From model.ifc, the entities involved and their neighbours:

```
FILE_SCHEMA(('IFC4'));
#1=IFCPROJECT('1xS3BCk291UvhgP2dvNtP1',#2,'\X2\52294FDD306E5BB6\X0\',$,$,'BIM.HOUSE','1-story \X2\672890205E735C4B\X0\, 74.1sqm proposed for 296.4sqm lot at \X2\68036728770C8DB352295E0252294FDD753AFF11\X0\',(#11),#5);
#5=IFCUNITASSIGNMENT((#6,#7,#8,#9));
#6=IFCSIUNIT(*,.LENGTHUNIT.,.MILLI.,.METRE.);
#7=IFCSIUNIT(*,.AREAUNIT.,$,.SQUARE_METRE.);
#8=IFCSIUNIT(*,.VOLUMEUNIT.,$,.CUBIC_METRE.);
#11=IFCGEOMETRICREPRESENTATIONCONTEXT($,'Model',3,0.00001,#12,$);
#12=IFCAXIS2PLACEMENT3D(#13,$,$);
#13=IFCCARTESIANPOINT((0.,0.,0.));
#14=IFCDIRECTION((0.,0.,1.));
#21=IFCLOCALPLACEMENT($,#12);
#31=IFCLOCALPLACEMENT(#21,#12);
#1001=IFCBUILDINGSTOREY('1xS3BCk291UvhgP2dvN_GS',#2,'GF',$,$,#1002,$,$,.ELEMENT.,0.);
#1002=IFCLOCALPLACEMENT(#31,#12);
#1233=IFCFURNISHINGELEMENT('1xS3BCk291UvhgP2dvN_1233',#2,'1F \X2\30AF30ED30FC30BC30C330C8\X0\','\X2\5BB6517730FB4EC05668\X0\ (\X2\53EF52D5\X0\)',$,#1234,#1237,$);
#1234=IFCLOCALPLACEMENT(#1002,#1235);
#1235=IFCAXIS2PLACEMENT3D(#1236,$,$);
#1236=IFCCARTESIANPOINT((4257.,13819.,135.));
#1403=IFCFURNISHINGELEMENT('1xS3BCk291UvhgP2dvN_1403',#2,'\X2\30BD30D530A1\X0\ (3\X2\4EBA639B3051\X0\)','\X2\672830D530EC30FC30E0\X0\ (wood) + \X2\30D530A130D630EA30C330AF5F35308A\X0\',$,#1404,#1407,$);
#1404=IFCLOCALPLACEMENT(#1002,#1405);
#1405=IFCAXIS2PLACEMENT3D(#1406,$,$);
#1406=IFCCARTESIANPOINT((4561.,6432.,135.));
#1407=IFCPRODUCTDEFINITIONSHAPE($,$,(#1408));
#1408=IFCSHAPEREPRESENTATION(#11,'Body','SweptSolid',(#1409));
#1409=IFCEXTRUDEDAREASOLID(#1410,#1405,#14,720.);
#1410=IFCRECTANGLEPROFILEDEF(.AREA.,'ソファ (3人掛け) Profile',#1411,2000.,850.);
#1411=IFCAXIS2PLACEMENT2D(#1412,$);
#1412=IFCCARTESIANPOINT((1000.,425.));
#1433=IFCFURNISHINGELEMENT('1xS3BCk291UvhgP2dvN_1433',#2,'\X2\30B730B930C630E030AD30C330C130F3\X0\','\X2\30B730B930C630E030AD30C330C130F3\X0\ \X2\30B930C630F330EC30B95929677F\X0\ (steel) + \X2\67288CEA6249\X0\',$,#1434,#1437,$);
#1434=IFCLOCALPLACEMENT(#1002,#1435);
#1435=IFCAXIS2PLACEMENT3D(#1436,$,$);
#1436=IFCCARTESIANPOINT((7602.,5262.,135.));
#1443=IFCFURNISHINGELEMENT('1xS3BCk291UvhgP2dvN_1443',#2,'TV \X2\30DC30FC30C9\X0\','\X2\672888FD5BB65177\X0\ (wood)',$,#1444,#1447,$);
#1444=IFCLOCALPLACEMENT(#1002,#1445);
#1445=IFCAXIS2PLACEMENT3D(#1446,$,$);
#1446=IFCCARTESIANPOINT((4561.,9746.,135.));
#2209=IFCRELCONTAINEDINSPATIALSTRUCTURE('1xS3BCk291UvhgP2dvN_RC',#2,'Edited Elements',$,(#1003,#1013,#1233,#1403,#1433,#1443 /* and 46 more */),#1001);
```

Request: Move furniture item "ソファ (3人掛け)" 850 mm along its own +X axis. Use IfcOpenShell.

```python
import ifcopenshell
import ifcopenshell.api.geometry
import ifcopenshell.util.placement
import ifcopenshell.util.unit

model = ifcopenshell.open("model.ifc")
unit_scale = ifcopenshell.util.unit.calculate_unit_scale(model)

item = model.by_guid("1xS3BCk291UvhgP2dvN_1403")
matrix = ifcopenshell.util.placement.get_local_placement(item.ObjectPlacement)
matrix[:3, 3] += matrix[:3, 0] * 0.85 / unit_scale
ifcopenshell.api.geometry.edit_object_placement(model, product=item, matrix=matrix, is_si=False)

print(ifcopenshell.util.placement.get_local_placement(item.ObjectPlacement).round(3) + 0.0)

model.write("model_v2.ifc")
```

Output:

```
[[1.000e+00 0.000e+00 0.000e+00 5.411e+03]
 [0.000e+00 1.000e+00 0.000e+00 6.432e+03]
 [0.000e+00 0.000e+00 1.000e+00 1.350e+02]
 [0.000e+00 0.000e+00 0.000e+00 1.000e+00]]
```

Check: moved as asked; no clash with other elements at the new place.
